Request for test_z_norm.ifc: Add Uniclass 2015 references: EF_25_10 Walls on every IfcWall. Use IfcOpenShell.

First a look at what the model holds.

```python
import ifcopenshell

model = ifcopenshell.open("test_z_norm.ifc")
print(model.schema)
print("classifications:", [c.Name for c in model.by_type("IfcClassification")])
for ifc_class in ("IfcDoor", "IfcRoof", "IfcStair", "IfcWall", "IfcWindow"):
    print(ifc_class, len(model.by_type(ifc_class)))
```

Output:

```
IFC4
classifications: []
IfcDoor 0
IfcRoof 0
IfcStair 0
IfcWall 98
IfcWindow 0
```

```python
import ifcopenshell
import ifcopenshell.api.classification

model = ifcopenshell.open("test_z_norm.ifc")

system = ifcopenshell.api.classification.add_classification(model, classification="Uniclass 2015")

codes = {
    "IfcWall": ("EF_25_10", "Walls"),
}
for ifc_class, (code, name) in codes.items():
    products = model.by_type(ifc_class)
    ifcopenshell.api.classification.add_reference(
        model, products=products, classification=system, identification=code, name=name
    )
    print(code, len(products))

model.write("test_z_norm_updated.ifc")
```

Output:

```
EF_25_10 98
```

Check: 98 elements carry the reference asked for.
